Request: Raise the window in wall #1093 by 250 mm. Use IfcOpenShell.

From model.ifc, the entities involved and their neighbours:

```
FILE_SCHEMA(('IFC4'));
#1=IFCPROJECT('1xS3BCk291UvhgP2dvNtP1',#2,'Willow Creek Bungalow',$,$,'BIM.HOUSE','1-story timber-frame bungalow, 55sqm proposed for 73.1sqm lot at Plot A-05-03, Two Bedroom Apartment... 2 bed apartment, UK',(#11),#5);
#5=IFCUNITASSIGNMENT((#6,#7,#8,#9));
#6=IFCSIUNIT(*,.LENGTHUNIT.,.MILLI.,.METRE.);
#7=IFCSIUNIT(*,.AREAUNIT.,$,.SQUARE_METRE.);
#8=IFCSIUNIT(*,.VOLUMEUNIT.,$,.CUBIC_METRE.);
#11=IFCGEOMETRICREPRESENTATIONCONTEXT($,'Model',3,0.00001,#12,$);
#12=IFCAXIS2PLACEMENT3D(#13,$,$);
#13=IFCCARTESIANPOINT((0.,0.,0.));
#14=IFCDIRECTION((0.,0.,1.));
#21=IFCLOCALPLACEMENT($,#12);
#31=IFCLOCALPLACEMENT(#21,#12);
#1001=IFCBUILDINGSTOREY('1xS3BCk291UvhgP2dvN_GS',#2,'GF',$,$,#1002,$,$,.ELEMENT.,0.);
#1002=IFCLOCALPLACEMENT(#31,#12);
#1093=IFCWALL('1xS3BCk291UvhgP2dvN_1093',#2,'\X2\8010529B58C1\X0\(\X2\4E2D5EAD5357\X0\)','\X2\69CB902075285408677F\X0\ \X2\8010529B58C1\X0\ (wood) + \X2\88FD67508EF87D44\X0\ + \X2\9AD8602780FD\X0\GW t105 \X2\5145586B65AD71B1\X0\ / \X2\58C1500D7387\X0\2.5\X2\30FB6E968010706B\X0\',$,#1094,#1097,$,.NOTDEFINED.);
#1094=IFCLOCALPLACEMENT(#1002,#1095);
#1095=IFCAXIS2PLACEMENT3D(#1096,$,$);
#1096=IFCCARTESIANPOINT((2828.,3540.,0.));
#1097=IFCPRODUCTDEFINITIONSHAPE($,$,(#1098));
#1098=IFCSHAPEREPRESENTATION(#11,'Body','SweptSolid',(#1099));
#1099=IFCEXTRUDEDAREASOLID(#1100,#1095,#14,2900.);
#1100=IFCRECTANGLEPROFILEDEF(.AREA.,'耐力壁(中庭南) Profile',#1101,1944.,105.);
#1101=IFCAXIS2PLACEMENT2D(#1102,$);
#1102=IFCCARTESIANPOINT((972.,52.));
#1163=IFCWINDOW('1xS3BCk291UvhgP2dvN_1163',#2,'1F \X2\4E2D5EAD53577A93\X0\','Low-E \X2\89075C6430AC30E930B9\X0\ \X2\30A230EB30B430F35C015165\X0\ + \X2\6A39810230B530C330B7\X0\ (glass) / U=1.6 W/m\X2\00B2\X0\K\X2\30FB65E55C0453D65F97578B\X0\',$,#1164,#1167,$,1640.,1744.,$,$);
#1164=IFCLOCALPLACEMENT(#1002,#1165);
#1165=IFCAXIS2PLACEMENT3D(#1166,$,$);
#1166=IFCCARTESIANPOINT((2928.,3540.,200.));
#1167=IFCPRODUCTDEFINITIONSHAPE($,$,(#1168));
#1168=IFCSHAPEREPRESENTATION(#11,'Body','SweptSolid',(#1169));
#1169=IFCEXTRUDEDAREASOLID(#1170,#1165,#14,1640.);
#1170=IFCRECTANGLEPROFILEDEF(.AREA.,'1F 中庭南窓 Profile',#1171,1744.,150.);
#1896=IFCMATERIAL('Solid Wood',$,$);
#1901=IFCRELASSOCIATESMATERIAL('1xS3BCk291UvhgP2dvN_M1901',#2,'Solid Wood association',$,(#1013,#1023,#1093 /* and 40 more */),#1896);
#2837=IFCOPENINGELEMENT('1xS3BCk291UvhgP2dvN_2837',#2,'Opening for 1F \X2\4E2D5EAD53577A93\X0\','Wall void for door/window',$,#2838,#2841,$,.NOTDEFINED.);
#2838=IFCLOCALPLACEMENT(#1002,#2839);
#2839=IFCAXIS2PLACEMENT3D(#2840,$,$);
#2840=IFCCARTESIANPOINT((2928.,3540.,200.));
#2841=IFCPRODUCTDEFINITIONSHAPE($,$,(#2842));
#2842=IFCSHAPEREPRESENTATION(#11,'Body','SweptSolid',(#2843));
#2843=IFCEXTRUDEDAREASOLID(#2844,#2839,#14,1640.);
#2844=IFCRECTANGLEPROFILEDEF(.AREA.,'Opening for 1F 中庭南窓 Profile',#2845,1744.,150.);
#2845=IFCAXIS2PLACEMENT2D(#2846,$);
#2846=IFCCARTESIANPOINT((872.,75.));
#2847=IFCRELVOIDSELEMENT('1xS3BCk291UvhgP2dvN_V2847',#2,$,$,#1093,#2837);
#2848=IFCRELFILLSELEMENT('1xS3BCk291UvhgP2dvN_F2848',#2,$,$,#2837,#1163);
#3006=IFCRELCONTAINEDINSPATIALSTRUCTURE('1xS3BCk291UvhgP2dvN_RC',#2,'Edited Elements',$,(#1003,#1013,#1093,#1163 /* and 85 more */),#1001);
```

```python
import numpy as np
import ifcopenshell
import ifcopenshell.api.geometry
import ifcopenshell.util.placement
import ifcopenshell.util.unit

model = ifcopenshell.open("model.ifc")
unit_scale = ifcopenshell.util.unit.calculate_unit_scale(model)

window = model.by_guid("1xS3BCk291UvhgP2dvN_1163")
opening = window.FillsVoids[0].RelatingOpeningElement
dz = 0.25 / unit_scale

shift = np.array([0.0, 0.0, dz])
# The window is not placed relative to its opening, so move both.
for product in (opening, window):
    matrix = ifcopenshell.util.placement.get_local_placement(product.ObjectPlacement)
    matrix[:3, 3] += shift
    ifcopenshell.api.geometry.edit_object_placement(model, product=product, matrix=matrix, is_si=False)

print(f"moved by {dz * unit_scale:+.3f} m")

model.write("model_edited.ifc")
```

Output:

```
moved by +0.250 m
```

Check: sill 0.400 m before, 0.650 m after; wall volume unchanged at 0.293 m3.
